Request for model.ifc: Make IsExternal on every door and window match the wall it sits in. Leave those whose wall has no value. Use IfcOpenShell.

First a look at what the model holds.

```python
import ifcopenshell
import ifcopenshell.util.element

model = ifcopenshell.open("model.ifc")
print(model.schema)
seen = {}
for e in model.by_type("IfcDoor") + model.by_type("IfcWindow"):
    if not e.FillsVoids:
        continue
    host = e.FillsVoids[0].RelatingOpeningElement.VoidsElements[0].RelatingBuildingElement
    own = ifcopenshell.util.element.get_pset(e, f"Pset_{e.is_a()[3:].removesuffix('StandardCase')}Common", "IsExternal")
    wall = ifcopenshell.util.element.get_pset(host, "Pset_WallCommon", "IsExternal")
    seen[e.is_a(), own, wall] = seen.get((e.is_a(), own, wall), 0) + 1
for (cls, own, wall), count in sorted(seen.items(), key=str):
    print(count, cls, "IsExternal:", own, "| host wall:", wall)
```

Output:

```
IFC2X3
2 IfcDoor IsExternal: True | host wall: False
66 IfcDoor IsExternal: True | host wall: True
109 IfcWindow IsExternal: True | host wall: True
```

```python
import ifcopenshell
import ifcopenshell.api.pset
import ifcopenshell.util.element

model = ifcopenshell.open("model.ifc")

count = 0
for ifc_class, pset_name in (("IfcDoor", "Pset_DoorCommon"), ("IfcWindow", "Pset_WindowCommon")):
    for e in model.by_type(ifc_class):
        if not e.FillsVoids:
            continue
        host = e.FillsVoids[0].RelatingOpeningElement.VoidsElements[0].RelatingBuildingElement
        external = ifcopenshell.util.element.get_pset(host, "Pset_WallCommon", "IsExternal")
        if external is None or ifcopenshell.util.element.get_pset(e, pset_name, "IsExternal") == external:
            continue
        pset = ifcopenshell.api.pset.add_pset(model, product=e, name=pset_name)
        ifcopenshell.api.pset.edit_pset(model, pset=pset, properties={"IsExternal": external})
        count += 1

print(count, "updated")

model.write("model_updated.ifc")
```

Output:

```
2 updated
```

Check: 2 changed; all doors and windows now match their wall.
